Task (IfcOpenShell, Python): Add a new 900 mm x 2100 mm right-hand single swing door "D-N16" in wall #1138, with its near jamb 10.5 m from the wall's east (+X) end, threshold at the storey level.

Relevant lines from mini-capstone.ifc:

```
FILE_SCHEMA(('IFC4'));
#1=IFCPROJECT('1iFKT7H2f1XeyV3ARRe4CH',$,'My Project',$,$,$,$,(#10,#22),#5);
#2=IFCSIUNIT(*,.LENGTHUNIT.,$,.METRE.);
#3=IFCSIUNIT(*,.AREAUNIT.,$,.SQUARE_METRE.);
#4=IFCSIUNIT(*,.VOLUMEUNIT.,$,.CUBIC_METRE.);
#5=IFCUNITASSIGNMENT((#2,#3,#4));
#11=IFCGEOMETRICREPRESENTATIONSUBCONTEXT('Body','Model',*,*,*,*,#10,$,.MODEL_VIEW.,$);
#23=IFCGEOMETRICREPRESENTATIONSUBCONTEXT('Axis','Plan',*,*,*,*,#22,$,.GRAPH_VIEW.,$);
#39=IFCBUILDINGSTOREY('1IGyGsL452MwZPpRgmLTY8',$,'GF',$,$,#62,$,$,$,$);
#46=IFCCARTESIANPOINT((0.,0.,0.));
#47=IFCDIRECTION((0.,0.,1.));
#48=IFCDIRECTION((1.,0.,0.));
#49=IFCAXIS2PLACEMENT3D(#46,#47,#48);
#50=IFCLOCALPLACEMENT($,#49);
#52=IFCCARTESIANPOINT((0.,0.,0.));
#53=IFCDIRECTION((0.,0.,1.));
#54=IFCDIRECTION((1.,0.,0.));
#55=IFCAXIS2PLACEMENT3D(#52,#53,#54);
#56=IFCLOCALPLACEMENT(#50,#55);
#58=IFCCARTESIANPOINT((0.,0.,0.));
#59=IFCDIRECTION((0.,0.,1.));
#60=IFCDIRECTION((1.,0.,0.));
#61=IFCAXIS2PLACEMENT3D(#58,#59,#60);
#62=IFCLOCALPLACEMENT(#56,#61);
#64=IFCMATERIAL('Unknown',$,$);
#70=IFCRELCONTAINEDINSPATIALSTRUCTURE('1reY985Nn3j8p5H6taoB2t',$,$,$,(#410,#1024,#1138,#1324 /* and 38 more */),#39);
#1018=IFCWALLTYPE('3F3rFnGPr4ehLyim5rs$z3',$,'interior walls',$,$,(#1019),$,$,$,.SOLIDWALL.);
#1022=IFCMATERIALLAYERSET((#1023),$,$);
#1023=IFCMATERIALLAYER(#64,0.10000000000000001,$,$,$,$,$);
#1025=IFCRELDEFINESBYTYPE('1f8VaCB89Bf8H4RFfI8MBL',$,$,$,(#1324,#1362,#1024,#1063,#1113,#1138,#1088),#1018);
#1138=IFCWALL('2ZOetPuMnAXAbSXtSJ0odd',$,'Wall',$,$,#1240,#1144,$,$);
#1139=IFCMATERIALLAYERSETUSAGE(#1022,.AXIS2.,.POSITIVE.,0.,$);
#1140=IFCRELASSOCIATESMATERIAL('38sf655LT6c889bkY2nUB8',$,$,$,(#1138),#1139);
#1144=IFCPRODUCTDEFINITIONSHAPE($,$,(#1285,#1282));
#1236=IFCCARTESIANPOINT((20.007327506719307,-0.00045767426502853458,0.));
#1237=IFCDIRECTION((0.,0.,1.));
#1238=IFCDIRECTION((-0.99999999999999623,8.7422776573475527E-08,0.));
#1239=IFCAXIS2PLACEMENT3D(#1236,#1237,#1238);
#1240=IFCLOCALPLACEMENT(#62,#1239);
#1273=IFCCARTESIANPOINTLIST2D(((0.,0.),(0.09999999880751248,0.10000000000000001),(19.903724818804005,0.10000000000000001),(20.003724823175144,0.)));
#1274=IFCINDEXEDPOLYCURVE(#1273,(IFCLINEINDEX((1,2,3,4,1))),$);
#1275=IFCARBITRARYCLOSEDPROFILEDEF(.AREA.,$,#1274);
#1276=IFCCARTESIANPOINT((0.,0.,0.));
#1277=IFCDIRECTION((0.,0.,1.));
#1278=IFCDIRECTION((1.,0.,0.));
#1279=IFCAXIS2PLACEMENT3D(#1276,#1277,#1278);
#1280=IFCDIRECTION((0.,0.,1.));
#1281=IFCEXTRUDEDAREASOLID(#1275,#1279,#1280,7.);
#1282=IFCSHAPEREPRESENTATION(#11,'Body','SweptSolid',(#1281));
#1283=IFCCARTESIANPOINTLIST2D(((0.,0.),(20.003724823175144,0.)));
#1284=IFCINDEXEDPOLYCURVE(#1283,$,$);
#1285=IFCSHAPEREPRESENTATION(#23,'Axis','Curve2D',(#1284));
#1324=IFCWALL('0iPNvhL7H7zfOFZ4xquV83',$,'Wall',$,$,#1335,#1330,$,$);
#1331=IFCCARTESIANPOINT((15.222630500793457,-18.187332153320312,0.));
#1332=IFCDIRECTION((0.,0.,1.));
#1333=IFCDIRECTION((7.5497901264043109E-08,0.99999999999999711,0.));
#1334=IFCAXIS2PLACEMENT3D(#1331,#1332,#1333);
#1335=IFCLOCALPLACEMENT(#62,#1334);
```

```python
import numpy as np
import ifcopenshell
import ifcopenshell.api.feature
import ifcopenshell.api.geometry
import ifcopenshell.api.root
import ifcopenshell.api.spatial
import ifcopenshell.geom
import ifcopenshell.util.element
import ifcopenshell.util.placement
import ifcopenshell.util.representation
import ifcopenshell.util.shape
import ifcopenshell.util.unit

model = ifcopenshell.open("mini-capstone.ifc")
unit_scale = ifcopenshell.util.unit.calculate_unit_scale(model)
settings = ifcopenshell.geom.settings()


def volume(element):
    """Net volume in cubic metres, openings subtracted."""
    shape = ifcopenshell.geom.create_shape(settings, element)
    return ifcopenshell.util.shape.get_volume(shape.geometry)


wall = model.by_guid("2ZOetPuMnAXAbSXtSJ0odd")
storey = ifcopenshell.util.element.get_container(wall, ifc_class="IfcBuildingStorey")
context = ifcopenshell.util.representation.get_context(model, "Model", "Body", "MODEL_VIEW")
before = volume(wall)

width, height, from_end, sill = 0.9, 2.1, 10.5, 0.0  # metres

# The wall runs along its own X axis, and the end named is its -X end.
wall_shape = ifcopenshell.geom.create_shape(settings, wall)
x, y, z = ifcopenshell.util.shape.get_vertices(wall_shape.geometry).T
start = x.min() + from_end
face, thickness = float(y.min()), float(y.max() - y.min())
wall_matrix = ifcopenshell.util.placement.get_local_placement(wall.ObjectPlacement)
level = ifcopenshell.util.placement.get_local_placement(storey.ObjectPlacement)[2, 3]


def in_wall(x, y):
    """Placement at x, y metres in the wall's axes, at sill height."""
    matrix = wall_matrix.copy()
    matrix[:, 3] = wall_matrix @ np.array([x / unit_scale, y / unit_scale, 0.0, 1.0])
    matrix[2, 3] = level + sill / unit_scale
    return matrix


# Opening: a box that overshoots both wall faces by 50 mm.
opening = ifcopenshell.api.root.create_entity(model, ifc_class="IfcOpeningElement", predefined_type="OPENING")
box = ifcopenshell.api.geometry.add_wall_representation(
    model, context=context, length=width, height=height, thickness=thickness + 0.1
)
ifcopenshell.api.geometry.assign_representation(model, product=opening, representation=box)
ifcopenshell.api.geometry.edit_object_placement(model, product=opening, matrix=in_wall(start, face - 0.05), is_si=False)
ifcopenshell.api.feature.add_feature(model, feature=opening, element=wall)

door = ifcopenshell.api.root.create_entity(model, ifc_class="IfcDoor", name="D-N16", predefined_type="DOOR")
door.OverallWidth, door.OverallHeight = width / unit_scale, height / unit_scale
door.OperationType = "SINGLE_SWING_RIGHT"
body = ifcopenshell.api.geometry.add_door_representation(
    model,
    context=context,
    overall_width=door.OverallWidth,
    overall_height=door.OverallHeight,
    operation_type="SINGLE_SWING_RIGHT",
    lining_properties={"LiningDepth": thickness / unit_scale, "ThresholdDepth": thickness / unit_scale},
)
ifcopenshell.api.geometry.assign_representation(model, product=door, representation=body)
ifcopenshell.api.spatial.assign_container(model, products=[door], relating_structure=storey)
ifcopenshell.api.feature.add_filling(model, opening=opening, element=door)

# The lining spans the wall, so the door starts at the wall face.
ifcopenshell.api.geometry.edit_object_placement(model, product=door, matrix=in_wall(start, face), is_si=False)

after = volume(wall)

print(f"wall volume {before:.3f} -> {after:.3f} m3")

model.write("mini-capstone_edited.ifc")
```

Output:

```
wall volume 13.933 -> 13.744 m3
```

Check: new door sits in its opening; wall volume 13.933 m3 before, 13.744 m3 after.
